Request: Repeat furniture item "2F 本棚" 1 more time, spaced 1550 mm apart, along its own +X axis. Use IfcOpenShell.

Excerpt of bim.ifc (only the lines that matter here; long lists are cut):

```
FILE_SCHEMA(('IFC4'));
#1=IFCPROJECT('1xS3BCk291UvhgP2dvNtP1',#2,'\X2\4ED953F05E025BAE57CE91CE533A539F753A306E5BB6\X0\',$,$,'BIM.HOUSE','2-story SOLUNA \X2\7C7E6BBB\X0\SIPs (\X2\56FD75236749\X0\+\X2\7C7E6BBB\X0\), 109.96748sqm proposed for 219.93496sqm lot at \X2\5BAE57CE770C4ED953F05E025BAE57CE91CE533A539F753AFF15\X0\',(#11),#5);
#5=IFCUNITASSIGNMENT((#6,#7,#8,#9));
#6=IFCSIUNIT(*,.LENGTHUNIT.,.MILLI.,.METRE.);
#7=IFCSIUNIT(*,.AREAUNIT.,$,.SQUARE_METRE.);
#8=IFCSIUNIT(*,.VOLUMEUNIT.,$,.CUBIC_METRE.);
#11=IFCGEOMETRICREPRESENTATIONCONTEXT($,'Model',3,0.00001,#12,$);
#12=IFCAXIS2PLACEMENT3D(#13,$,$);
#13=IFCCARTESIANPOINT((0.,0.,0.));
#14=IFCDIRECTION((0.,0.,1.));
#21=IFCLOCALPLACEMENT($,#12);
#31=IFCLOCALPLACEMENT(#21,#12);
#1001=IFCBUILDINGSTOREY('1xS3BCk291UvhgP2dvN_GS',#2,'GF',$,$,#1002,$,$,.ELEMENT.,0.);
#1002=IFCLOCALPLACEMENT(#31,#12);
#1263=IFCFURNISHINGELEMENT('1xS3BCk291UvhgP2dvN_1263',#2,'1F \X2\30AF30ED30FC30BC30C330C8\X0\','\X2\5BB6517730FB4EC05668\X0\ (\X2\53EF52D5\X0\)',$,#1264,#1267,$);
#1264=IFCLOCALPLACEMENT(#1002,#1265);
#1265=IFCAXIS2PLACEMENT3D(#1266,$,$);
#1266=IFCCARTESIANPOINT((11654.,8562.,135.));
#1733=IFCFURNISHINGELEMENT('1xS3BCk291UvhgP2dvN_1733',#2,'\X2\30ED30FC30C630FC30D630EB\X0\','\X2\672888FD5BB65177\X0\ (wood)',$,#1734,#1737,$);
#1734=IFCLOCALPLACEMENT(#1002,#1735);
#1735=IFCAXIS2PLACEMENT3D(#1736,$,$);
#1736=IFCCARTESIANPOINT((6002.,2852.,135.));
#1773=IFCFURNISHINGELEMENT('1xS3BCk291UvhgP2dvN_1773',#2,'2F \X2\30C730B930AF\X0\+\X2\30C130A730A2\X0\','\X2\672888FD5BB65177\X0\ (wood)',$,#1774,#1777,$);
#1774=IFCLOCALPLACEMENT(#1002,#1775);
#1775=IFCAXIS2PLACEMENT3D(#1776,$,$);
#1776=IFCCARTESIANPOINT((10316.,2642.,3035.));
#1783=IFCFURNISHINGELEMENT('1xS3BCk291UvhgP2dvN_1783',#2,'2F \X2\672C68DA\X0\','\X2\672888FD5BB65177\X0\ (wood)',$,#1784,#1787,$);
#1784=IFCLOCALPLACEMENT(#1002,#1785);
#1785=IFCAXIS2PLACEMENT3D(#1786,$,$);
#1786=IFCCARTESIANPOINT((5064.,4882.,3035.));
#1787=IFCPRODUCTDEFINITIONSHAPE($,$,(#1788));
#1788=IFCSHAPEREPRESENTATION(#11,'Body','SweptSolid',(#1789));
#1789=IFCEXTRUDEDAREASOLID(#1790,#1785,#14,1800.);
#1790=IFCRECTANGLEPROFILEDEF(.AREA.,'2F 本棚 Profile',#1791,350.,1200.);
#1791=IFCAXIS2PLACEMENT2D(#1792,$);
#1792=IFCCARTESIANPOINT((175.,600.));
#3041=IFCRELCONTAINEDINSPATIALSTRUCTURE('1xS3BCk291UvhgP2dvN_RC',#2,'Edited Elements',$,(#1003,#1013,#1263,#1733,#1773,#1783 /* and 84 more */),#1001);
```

```python
import ifcopenshell
import ifcopenshell.api.geometry
import ifcopenshell.api.root
import ifcopenshell.util.element
import ifcopenshell.util.placement
import ifcopenshell.util.unit

model = ifcopenshell.open("bim.ifc")
unit_scale = ifcopenshell.util.unit.calculate_unit_scale(model)


def reuse_history(source, copy):
    """copy_class also copies each property set's owner history, people and application; keep the originals."""
    for rel in copy.IsDefinedBy:
        if rel.is_a("IfcRelDefinesByProperties") and (history := rel.RelatingPropertyDefinition.OwnerHistory):
            rel.RelatingPropertyDefinition.OwnerHistory = source.OwnerHistory
            ifcopenshell.util.element.remove_deep2(model, history)


source = model.by_guid("1xS3BCk291UvhgP2dvN_1783")
base = ifcopenshell.util.placement.get_local_placement(source.ObjectPlacement)
step = base[:3, 0] * 1.55 / unit_scale

for i in range(1, 2):
    copy = ifcopenshell.api.root.copy_class(model, product=source)
    copy.Representation = ifcopenshell.util.element.copy_deep(
        model, source.Representation, exclude=["IfcGeometricRepresentationContext", "IfcRepresentationMap"]
    )
    reuse_history(source, copy)
    matrix = base.copy()
    matrix[:3, 3] += i * step
    print("added at", matrix[:3, 3].round(3) + 0.0)
    ifcopenshell.api.geometry.edit_object_placement(model, product=copy, matrix=matrix, is_si=False)

model.write("bim_rev.ifc")
```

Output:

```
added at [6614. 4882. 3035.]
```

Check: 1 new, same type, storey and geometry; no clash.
